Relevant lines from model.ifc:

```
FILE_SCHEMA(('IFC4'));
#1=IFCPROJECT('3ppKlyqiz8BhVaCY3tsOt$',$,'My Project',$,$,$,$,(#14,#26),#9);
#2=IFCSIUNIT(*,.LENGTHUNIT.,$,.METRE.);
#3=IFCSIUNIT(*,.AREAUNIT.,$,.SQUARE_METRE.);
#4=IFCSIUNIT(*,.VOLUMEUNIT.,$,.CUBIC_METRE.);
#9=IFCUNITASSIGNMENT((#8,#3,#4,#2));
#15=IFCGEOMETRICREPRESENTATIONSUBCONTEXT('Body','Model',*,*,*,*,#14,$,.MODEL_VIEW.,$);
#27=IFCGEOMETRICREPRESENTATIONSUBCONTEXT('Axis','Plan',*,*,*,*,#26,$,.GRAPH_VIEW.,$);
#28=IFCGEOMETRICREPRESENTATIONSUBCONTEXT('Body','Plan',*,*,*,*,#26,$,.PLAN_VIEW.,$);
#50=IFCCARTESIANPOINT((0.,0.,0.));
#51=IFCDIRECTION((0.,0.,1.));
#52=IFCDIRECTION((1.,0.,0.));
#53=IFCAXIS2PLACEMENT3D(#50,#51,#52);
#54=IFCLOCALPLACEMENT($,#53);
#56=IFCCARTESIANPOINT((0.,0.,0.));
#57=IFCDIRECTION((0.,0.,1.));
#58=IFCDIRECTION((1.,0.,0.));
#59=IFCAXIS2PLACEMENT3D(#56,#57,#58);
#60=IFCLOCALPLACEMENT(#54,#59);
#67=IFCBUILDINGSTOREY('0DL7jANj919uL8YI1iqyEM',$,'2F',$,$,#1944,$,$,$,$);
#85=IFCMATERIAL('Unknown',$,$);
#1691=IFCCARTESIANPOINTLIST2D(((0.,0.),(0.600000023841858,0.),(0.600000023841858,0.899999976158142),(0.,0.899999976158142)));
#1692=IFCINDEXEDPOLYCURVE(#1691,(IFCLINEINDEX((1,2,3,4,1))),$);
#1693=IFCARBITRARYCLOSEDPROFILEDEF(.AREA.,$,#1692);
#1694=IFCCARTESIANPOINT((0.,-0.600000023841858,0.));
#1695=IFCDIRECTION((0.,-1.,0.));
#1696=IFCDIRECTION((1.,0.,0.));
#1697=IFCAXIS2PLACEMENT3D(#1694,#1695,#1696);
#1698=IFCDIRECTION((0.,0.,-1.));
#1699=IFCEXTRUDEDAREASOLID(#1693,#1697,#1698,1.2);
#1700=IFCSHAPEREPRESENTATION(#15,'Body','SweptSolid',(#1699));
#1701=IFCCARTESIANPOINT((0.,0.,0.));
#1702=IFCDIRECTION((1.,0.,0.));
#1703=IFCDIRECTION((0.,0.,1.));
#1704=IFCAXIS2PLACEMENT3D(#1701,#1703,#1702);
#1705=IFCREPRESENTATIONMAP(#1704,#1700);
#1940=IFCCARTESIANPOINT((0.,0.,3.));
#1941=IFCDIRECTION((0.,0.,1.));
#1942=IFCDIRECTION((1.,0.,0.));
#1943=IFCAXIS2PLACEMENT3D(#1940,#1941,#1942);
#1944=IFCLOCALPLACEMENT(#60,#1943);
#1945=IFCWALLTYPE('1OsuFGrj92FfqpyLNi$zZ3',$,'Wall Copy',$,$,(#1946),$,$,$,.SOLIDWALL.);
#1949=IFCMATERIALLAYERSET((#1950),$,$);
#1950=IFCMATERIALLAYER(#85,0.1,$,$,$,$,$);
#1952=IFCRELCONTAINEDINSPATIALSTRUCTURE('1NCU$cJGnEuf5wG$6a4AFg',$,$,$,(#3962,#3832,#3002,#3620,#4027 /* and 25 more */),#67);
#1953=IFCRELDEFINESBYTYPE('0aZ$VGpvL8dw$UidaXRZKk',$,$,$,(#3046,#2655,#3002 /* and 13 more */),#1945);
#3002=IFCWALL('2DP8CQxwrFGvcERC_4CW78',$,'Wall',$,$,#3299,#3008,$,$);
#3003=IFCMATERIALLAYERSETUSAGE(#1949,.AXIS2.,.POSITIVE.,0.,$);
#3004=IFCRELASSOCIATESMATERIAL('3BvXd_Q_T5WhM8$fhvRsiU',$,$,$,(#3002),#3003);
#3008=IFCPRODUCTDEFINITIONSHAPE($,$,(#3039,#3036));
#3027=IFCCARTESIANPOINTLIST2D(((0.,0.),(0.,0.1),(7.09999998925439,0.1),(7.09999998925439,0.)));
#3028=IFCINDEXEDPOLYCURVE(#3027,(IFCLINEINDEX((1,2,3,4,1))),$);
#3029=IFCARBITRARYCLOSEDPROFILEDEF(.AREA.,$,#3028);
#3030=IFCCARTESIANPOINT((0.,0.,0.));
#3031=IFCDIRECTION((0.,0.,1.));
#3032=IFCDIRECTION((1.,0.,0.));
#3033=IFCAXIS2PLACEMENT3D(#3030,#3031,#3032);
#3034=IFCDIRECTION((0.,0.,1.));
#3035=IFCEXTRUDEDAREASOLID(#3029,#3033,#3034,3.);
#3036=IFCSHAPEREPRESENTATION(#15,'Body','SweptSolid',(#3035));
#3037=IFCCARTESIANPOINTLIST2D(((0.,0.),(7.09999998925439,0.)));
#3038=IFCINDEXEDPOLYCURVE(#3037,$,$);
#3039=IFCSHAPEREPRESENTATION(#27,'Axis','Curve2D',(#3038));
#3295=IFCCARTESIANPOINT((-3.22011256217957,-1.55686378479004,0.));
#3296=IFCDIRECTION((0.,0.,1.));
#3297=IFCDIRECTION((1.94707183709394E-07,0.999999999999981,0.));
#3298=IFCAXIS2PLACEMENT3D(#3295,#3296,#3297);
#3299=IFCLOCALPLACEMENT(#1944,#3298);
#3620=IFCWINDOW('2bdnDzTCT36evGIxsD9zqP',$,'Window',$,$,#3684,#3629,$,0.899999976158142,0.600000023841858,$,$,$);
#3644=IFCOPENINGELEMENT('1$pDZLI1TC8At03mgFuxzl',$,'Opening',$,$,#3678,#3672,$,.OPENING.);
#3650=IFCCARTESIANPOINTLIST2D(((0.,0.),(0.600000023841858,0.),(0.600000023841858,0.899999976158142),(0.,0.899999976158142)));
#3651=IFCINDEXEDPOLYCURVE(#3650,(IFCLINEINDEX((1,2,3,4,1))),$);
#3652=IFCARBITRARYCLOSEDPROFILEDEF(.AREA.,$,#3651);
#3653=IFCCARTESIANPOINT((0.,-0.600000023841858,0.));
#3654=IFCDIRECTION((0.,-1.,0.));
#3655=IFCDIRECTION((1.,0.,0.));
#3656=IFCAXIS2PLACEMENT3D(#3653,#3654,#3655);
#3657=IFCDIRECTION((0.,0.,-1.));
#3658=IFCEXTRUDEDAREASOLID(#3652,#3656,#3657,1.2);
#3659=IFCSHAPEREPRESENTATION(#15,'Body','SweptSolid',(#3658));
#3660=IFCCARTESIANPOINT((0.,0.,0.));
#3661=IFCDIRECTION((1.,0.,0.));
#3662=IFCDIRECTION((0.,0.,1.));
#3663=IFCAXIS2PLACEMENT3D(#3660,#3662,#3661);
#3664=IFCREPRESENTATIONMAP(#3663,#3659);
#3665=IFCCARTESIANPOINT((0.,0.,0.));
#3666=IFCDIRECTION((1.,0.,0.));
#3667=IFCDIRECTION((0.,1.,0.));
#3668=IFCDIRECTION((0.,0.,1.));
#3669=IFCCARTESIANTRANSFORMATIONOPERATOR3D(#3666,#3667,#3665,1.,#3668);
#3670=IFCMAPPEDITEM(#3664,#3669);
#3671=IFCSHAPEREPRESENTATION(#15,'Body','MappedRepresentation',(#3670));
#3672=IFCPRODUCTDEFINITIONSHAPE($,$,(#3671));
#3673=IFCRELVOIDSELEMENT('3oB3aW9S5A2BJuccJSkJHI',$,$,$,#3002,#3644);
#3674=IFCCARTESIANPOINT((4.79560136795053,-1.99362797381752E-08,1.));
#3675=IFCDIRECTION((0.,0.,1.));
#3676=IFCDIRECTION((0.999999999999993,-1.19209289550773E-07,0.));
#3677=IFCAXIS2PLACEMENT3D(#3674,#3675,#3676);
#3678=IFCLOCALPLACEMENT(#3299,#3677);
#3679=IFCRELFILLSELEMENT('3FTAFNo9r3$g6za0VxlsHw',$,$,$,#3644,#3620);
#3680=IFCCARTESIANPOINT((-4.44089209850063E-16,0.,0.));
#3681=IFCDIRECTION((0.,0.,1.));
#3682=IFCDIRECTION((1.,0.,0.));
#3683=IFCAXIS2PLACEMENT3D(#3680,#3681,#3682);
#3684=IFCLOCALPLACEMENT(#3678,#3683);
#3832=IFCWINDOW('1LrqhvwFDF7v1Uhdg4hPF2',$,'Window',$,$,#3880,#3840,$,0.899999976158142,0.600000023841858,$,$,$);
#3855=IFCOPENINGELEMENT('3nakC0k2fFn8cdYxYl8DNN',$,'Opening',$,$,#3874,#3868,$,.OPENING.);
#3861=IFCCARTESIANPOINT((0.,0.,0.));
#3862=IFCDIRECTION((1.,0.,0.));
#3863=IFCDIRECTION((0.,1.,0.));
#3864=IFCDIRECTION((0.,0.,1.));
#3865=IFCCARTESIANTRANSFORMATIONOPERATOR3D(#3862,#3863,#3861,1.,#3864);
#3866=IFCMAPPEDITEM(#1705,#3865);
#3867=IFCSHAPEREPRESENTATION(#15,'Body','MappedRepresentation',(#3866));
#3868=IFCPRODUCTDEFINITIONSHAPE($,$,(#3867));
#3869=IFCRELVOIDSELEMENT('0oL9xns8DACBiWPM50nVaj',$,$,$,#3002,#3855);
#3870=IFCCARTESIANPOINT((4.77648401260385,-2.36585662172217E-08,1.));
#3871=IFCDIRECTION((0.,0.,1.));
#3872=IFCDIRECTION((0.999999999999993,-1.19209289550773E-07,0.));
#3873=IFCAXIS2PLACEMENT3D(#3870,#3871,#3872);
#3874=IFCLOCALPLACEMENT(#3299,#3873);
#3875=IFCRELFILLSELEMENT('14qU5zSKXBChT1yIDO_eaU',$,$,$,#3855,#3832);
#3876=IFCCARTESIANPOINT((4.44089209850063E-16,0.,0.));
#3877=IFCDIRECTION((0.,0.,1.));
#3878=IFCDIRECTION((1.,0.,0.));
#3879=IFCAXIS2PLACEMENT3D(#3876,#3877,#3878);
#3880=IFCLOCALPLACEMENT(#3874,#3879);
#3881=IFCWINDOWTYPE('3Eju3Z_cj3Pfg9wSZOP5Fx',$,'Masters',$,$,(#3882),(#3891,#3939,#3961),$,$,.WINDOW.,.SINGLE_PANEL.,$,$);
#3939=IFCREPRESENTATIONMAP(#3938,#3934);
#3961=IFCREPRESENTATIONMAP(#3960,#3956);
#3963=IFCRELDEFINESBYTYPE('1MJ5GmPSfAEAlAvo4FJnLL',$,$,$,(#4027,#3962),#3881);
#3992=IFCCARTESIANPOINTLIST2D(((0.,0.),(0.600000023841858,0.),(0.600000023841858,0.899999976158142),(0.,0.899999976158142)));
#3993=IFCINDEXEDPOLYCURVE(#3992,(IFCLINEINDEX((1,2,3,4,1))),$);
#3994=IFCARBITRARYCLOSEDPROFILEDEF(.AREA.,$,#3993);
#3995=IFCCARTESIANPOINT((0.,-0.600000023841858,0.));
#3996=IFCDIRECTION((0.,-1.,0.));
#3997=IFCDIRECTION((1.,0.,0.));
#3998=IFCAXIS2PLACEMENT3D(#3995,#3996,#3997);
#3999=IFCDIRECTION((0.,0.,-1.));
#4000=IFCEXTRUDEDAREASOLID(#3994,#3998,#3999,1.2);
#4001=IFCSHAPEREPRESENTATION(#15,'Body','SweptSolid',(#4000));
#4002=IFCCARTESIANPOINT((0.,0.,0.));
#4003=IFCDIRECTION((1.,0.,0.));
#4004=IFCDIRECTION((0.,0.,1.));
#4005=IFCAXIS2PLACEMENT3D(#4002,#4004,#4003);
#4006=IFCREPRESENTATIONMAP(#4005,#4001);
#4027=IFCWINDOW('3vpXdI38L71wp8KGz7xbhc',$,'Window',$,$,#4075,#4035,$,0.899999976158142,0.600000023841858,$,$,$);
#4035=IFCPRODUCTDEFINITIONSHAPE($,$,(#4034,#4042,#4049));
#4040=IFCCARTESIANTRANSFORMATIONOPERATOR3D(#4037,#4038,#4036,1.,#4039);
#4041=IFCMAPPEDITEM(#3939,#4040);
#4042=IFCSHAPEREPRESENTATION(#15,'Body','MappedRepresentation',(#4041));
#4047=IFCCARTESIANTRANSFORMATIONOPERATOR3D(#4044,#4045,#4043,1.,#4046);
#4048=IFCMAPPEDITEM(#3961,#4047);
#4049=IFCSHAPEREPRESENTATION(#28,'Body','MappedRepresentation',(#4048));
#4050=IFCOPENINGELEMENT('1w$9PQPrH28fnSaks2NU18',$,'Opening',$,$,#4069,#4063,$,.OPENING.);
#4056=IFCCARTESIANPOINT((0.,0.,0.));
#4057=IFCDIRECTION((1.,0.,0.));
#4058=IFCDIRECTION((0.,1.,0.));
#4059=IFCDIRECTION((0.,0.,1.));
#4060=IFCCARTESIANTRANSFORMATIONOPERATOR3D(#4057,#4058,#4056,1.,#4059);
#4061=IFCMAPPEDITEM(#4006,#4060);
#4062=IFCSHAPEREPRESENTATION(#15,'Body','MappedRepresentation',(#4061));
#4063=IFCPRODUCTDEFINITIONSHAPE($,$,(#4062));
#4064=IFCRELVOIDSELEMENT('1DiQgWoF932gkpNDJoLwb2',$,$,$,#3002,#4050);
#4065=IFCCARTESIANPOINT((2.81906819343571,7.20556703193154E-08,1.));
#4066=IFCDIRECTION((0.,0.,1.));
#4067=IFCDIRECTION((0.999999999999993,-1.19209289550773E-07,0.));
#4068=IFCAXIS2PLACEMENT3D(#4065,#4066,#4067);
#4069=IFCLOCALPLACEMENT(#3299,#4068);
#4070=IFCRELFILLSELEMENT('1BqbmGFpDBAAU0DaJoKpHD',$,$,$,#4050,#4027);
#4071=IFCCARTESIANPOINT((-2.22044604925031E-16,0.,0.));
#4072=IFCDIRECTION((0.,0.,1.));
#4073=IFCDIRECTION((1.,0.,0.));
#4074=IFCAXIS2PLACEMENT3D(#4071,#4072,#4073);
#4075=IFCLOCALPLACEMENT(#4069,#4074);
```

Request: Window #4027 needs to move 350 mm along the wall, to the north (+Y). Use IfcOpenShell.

```python
import ifcopenshell
import ifcopenshell.api.geometry
import ifcopenshell.util.placement
import ifcopenshell.util.unit

model = ifcopenshell.open("model.ifc")
unit_scale = ifcopenshell.util.unit.calculate_unit_scale(model)

window = model.by_guid("3vpXdI38L71wp8KGz7xbhc")
opening = window.FillsVoids[0].RelatingOpeningElement
wall = opening.VoidsElements[0].RelatingBuildingElement

wall_matrix = ifcopenshell.util.placement.get_local_placement(wall.ObjectPlacement)
shift = wall_matrix[:3, 0] * 0.35 / unit_scale
before = ifcopenshell.util.placement.get_local_placement(window.ObjectPlacement)[:3, 3].copy()

# The window is placed relative to its opening, so it follows when the opening moves.
matrix = ifcopenshell.util.placement.get_local_placement(opening.ObjectPlacement)
matrix[:3, 3] += shift
ifcopenshell.api.geometry.edit_object_placement(
    model, product=opening, matrix=matrix, is_si=False, should_transform_children=True
)

after = ifcopenshell.util.placement.get_local_placement(window.ObjectPlacement)[:3, 3]
print("window moved by", (after - before).round(3) + 0.0)

model.write("model-out.ifc")
```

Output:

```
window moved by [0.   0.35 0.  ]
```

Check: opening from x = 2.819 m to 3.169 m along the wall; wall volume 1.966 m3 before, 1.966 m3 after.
